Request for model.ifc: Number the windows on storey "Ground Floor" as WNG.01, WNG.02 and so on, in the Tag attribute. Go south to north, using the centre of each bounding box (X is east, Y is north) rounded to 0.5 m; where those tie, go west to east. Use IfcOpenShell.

First a look at what the model holds.

```python
import ifcopenshell
import ifcopenshell.util.element
import ifcopenshell.util.placement

model = ifcopenshell.open("model.ifc")
print(model.schema)
storey = next(s for s in model.by_type("IfcBuildingStorey") if s.Name == "Ground Floor")
windows = [e for e in ifcopenshell.util.element.get_decomposition(storey) if e.is_a("IfcWindow")]
for e in sorted(windows, key=lambda e: e.id()):
    origin = ifcopenshell.util.placement.get_local_placement(e.ObjectPlacement)[:3, 3]
    print(e.id(), e.Tag, e.Name, origin.round(2) + 0.0, sep=" | ")
```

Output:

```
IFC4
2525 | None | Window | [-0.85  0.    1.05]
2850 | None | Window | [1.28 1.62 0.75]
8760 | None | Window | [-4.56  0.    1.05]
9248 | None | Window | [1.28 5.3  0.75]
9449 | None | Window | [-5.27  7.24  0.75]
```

```python
import ifcopenshell
import ifcopenshell.geom
import ifcopenshell.util.element
import ifcopenshell.util.shape

model = ifcopenshell.open("model.ifc")
settings = ifcopenshell.geom.settings()
settings.set("use-world-coords", True)


def centre(element):
    shape = ifcopenshell.geom.create_shape(settings, element)
    return ifcopenshell.util.shape.get_bbox_centroid(shape.geometry)


storey = next(s for s in model.by_type("IfcBuildingStorey") if s.Name == "Ground Floor")
windows = [e for e in ifcopenshell.util.element.get_decomposition(storey) if e.is_a("IfcWindow")]

# Insertion points can sit at a corner or the storey origin, so sort by the geometry (in metres).
centres = {e: centre(e) for e in windows}
windows.sort(key=lambda e: (round(centres[e][1] / 0.5), centres[e][0]))

for i, e in enumerate(windows, start=1):
    number = f"WNG.{i:02d}"
    e.Tag = number
    print(e.id(), number)

model.write("model_rev.ifc")
```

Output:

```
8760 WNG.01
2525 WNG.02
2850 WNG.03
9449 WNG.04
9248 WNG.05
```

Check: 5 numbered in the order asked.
